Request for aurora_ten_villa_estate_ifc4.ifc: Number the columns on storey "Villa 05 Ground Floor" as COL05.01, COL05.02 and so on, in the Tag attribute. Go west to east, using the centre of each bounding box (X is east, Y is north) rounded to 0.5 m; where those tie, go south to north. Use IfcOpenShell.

First a look at what the model holds.

```python
import ifcopenshell
import ifcopenshell.util.element
import ifcopenshell.util.placement

model = ifcopenshell.open("aurora_ten_villa_estate_ifc4.ifc")
print(model.schema)
storey = next(s for s in model.by_type("IfcBuildingStorey") if s.Name == "Villa 05 Ground Floor")
columns = [e for e in ifcopenshell.util.element.get_decomposition(storey) if e.is_a("IfcColumn")]
for e in sorted(columns, key=lambda e: e.id()):
    origin = ifcopenshell.util.placement.get_local_placement(e.ObjectPlacement)[:3, 3]
    print(e.id(), e.Tag, e.Name, origin.round(2) + 0.0, sep=" | ")
```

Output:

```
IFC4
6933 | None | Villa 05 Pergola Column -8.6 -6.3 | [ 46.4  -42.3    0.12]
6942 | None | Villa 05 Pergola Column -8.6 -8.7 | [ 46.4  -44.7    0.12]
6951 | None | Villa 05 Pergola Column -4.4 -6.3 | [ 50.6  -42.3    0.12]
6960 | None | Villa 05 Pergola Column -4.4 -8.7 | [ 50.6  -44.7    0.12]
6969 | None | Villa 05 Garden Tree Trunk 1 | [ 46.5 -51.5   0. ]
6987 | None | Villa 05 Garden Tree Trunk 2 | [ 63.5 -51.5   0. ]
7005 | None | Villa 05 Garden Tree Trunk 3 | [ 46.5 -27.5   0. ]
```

```python
import ifcopenshell
import ifcopenshell.geom
import ifcopenshell.util.element
import ifcopenshell.util.shape

model = ifcopenshell.open("aurora_ten_villa_estate_ifc4.ifc")
settings = ifcopenshell.geom.settings()
settings.set("use-world-coords", True)


def centre(element):
    shape = ifcopenshell.geom.create_shape(settings, element)
    return ifcopenshell.util.shape.get_bbox_centroid(shape.geometry)


storey = next(s for s in model.by_type("IfcBuildingStorey") if s.Name == "Villa 05 Ground Floor")
columns = [e for e in ifcopenshell.util.element.get_decomposition(storey) if e.is_a("IfcColumn")]

# Insertion points can sit at a corner or the storey origin, so sort by the geometry (in metres).
centres = {e: centre(e) for e in columns}
columns.sort(key=lambda e: (round(centres[e][0] / 0.5), centres[e][1]))

for i, e in enumerate(columns, start=1):
    number = f"COL05.{i:02d}"
    e.Tag = number
    print(e.id(), number)

model.write("aurora_ten_villa_estate_ifc4_v2.ifc")
```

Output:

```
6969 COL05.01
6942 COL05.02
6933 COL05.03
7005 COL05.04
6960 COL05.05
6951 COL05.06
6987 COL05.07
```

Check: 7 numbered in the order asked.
